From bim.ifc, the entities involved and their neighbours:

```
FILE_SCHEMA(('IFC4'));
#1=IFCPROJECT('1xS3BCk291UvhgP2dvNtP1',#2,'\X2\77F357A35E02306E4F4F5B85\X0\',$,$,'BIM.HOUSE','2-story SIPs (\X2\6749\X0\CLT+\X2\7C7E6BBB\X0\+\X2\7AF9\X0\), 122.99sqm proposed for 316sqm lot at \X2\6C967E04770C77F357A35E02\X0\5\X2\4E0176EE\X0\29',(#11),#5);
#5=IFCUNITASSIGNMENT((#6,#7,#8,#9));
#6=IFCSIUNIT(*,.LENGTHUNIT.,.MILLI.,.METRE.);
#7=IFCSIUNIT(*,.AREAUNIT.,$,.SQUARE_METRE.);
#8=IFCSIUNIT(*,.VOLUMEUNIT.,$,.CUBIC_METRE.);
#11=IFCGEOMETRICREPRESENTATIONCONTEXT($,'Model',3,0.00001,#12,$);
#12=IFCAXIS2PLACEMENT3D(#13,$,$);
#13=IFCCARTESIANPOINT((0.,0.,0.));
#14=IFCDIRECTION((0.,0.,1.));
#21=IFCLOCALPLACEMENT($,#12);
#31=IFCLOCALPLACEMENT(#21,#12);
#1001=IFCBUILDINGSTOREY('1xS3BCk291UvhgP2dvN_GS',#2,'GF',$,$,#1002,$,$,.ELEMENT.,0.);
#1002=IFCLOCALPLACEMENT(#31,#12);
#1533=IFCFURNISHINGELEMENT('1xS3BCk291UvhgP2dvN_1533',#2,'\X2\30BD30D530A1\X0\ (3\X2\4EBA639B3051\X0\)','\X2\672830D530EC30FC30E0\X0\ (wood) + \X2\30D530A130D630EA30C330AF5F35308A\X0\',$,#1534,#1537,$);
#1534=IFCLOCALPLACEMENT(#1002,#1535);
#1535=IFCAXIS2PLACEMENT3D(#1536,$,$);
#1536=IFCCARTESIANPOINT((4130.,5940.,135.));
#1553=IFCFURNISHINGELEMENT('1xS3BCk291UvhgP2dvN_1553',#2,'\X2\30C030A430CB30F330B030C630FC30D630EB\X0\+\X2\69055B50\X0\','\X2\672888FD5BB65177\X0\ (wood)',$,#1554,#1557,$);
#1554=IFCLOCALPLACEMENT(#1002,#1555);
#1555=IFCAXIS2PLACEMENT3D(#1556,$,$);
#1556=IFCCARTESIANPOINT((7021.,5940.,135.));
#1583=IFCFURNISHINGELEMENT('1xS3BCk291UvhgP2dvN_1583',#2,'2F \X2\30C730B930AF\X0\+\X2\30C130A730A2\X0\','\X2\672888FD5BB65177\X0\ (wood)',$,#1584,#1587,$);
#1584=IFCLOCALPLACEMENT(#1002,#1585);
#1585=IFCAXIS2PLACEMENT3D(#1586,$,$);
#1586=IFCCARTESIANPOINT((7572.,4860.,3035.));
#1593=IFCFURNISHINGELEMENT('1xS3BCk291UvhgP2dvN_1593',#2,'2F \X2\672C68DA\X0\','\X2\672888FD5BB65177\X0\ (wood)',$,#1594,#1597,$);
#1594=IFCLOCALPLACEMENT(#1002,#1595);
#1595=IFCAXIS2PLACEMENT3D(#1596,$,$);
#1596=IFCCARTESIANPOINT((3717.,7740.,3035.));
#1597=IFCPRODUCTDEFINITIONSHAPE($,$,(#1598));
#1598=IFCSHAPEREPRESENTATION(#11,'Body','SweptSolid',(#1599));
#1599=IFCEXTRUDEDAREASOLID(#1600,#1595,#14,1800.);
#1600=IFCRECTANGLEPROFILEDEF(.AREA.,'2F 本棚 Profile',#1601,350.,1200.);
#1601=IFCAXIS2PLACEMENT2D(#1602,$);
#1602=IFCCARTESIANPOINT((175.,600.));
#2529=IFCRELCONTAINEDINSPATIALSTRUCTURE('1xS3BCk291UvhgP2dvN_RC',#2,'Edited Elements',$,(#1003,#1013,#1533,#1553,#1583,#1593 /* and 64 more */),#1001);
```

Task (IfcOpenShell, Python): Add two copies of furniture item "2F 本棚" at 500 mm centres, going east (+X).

```python
import numpy as np
import ifcopenshell
import ifcopenshell.api.geometry
import ifcopenshell.api.root
import ifcopenshell.util.element
import ifcopenshell.util.placement
import ifcopenshell.util.unit

model = ifcopenshell.open("bim.ifc")
unit_scale = ifcopenshell.util.unit.calculate_unit_scale(model)


def reuse_history(source, copy):
    """copy_class also copies each property set's owner history, people and application; keep the originals."""
    for rel in copy.IsDefinedBy:
        if rel.is_a("IfcRelDefinesByProperties") and (history := rel.RelatingPropertyDefinition.OwnerHistory):
            rel.RelatingPropertyDefinition.OwnerHistory = source.OwnerHistory
            ifcopenshell.util.element.remove_deep2(model, history)


source = model.by_guid("1xS3BCk291UvhgP2dvN_1593")
base = ifcopenshell.util.placement.get_local_placement(source.ObjectPlacement)
step = np.array([1.0, 0.0, 0.0]) * 0.5 / unit_scale

for i in range(1, 3):
    copy = ifcopenshell.api.root.copy_class(model, product=source)
    copy.Representation = ifcopenshell.util.element.copy_deep(
        model, source.Representation, exclude=["IfcGeometricRepresentationContext", "IfcRepresentationMap"]
    )
    reuse_history(source, copy)
    matrix = base.copy()
    matrix[:3, 3] += i * step
    print("added at", matrix[:3, 3].round(3) + 0.0)
    ifcopenshell.api.geometry.edit_object_placement(model, product=copy, matrix=matrix, is_si=False)

model.write("bim_edited.ifc")
```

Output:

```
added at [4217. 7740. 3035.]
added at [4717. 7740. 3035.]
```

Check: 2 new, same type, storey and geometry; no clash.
